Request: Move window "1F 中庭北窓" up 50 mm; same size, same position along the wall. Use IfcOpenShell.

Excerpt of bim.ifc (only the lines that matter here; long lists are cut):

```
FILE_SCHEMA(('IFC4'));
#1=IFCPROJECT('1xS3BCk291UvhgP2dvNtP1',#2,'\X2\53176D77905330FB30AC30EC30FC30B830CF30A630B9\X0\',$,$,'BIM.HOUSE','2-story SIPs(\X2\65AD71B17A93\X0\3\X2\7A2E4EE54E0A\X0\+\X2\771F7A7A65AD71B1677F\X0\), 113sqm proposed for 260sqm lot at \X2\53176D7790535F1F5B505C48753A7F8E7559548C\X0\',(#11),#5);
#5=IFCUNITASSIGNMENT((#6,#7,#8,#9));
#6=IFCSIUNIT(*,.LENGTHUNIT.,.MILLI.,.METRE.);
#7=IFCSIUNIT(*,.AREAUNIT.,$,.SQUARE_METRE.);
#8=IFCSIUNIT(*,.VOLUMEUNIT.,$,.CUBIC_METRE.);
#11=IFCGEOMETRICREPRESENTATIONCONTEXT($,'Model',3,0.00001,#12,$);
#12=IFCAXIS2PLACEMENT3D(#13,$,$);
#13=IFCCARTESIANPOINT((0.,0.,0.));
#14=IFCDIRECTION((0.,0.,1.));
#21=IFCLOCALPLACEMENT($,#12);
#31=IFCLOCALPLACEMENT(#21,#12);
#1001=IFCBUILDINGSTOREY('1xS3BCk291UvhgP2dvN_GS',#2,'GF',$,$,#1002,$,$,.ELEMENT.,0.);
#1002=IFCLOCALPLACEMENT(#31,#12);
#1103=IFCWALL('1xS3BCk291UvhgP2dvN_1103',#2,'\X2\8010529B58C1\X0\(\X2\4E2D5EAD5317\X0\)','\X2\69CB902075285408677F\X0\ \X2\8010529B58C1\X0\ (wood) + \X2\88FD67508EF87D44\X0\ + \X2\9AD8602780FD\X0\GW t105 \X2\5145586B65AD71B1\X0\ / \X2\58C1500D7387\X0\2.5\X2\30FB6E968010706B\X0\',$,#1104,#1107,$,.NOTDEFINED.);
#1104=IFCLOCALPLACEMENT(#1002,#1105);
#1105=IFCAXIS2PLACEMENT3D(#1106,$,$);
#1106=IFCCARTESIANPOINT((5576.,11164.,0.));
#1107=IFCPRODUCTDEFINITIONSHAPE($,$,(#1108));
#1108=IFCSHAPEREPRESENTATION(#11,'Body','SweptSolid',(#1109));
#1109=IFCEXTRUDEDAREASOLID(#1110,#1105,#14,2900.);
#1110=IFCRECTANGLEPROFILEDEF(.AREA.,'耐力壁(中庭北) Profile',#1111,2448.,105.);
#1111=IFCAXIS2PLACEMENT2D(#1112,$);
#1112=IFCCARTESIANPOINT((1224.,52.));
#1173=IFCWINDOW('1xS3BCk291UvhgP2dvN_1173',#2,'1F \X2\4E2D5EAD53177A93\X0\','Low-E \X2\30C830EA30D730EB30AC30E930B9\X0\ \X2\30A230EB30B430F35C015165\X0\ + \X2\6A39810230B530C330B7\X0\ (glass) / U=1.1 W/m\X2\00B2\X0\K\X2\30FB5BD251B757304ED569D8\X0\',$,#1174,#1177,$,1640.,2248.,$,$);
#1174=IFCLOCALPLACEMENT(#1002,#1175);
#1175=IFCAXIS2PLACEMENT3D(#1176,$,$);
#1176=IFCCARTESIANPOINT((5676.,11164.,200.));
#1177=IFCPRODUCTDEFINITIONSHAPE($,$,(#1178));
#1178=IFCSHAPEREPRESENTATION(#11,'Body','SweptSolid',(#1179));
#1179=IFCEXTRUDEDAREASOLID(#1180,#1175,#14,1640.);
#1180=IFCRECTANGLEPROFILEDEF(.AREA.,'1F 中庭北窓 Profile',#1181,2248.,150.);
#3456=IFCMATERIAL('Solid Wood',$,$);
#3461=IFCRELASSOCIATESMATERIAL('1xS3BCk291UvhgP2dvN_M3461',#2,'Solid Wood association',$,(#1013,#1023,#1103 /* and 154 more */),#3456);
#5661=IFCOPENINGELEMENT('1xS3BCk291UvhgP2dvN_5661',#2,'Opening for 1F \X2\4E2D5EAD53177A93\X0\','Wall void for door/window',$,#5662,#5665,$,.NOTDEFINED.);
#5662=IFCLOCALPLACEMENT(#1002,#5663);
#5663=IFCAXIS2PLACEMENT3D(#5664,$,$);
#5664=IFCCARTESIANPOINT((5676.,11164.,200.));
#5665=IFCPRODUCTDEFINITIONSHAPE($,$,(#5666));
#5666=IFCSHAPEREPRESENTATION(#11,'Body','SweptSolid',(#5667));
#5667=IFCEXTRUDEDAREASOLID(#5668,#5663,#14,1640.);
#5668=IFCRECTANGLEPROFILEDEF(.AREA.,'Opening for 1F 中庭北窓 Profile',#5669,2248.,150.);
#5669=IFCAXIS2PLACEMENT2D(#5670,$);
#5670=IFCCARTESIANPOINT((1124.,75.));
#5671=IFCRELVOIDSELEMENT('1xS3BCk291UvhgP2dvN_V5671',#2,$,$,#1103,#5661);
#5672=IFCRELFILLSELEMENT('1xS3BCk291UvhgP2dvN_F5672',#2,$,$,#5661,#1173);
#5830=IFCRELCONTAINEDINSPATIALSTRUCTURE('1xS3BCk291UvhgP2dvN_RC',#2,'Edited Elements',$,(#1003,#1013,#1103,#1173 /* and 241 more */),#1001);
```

```python
import numpy as np
import ifcopenshell
import ifcopenshell.api.geometry
import ifcopenshell.util.placement
import ifcopenshell.util.unit

model = ifcopenshell.open("bim.ifc")
unit_scale = ifcopenshell.util.unit.calculate_unit_scale(model)

window = model.by_guid("1xS3BCk291UvhgP2dvN_1173")
opening = window.FillsVoids[0].RelatingOpeningElement
dz = 50.0

shift = np.array([0.0, 0.0, dz])
# The window is not placed relative to its opening, so move both.
for product in (opening, window):
    matrix = ifcopenshell.util.placement.get_local_placement(product.ObjectPlacement)
    matrix[:3, 3] += shift
    ifcopenshell.api.geometry.edit_object_placement(model, product=product, matrix=matrix, is_si=False)

print(f"moved by {dz * unit_scale:+.3f} m")

model.write("bim_updated.ifc")
```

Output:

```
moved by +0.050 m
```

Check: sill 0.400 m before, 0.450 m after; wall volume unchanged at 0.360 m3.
